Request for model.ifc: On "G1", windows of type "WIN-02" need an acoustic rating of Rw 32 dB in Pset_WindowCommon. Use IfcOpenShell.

First a look at what the model holds.

```python
import ifcopenshell
import ifcopenshell.util.element

model = ifcopenshell.open("model.ifc")
print(model.schema)
storey = next(s for s in model.by_type("IfcBuildingStorey") if s.Name == "G1")
windows = [e for e in ifcopenshell.util.element.get_decomposition(storey) if e.is_a("IfcWindow")]
seen = {}
for e in windows:
    element_type = ifcopenshell.util.element.get_type(e)
    key = (element_type.Name if element_type != e and element_type else None, ifcopenshell.util.element.get_pset(e, "Pset_WindowCommon", "AcousticRating"))
    seen[key] = seen.get(key, 0) + 1
for (name, value), count in sorted(seen.items(), key=str):
    print(count, "x", name, "|", value)
```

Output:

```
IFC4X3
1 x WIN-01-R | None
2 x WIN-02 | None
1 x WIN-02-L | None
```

```python
import ifcopenshell
import ifcopenshell.api.pset
import ifcopenshell.util.element

model = ifcopenshell.open("model.ifc")

storey = next(s for s in model.by_type("IfcBuildingStorey") if s.Name == "G1")
windows = [e for e in ifcopenshell.util.element.get_decomposition(storey) if e.is_a("IfcWindow")]

count = 0
for e in windows:
    element_type = ifcopenshell.util.element.get_type(e)
    if element_type in (None, e) or element_type.Name != "WIN-02":
        continue
    # add_pset returns the element's existing set when there is one.
    pset = ifcopenshell.api.pset.add_pset(model, product=e, name="Pset_WindowCommon")
    ifcopenshell.api.pset.edit_pset(model, pset=pset, properties={"AcousticRating": "Rw 32 dB"})
    count += 1

print(count, "windows updated")

model.write("model_rev.ifc")
```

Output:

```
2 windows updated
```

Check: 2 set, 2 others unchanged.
